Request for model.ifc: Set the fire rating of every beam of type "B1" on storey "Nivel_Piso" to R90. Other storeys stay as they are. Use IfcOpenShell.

First a look at what the model holds.

```python
import ifcopenshell
import ifcopenshell.util.element

model = ifcopenshell.open("model.ifc")
print(model.schema)
storey = next(s for s in model.by_type("IfcBuildingStorey") if s.Name == "Nivel_Piso")
beams = [e for e in ifcopenshell.util.element.get_decomposition(storey) if e.is_a("IfcBeam")]
seen = {}
for e in beams:
    element_type = ifcopenshell.util.element.get_type(e)
    key = (element_type.Name if element_type != e and element_type else None, ifcopenshell.util.element.get_pset(e, "Pset_BeamCommon", "FireRating"))
    seen[key] = seen.get(key, 0) + 1
for (name, value), count in sorted(seen.items(), key=str):
    print(count, "x", name, "|", value)
```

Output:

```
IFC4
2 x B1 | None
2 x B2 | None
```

```python
import ifcopenshell
import ifcopenshell.api.pset
import ifcopenshell.util.element

model = ifcopenshell.open("model.ifc")

storey = next(s for s in model.by_type("IfcBuildingStorey") if s.Name == "Nivel_Piso")
beams = [e for e in ifcopenshell.util.element.get_decomposition(storey) if e.is_a("IfcBeam")]

count = 0
for e in beams:
    element_type = ifcopenshell.util.element.get_type(e)
    if element_type in (None, e) or element_type.Name != "B1":
        continue
    # add_pset returns the element's existing set when there is one.
    pset = ifcopenshell.api.pset.add_pset(model, product=e, name="Pset_BeamCommon")
    ifcopenshell.api.pset.edit_pset(model, pset=pset, properties={"FireRating": "R90"})
    count += 1

print(count, "beams updated")

model.write("model_v2.ifc")
```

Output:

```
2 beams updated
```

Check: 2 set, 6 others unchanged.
